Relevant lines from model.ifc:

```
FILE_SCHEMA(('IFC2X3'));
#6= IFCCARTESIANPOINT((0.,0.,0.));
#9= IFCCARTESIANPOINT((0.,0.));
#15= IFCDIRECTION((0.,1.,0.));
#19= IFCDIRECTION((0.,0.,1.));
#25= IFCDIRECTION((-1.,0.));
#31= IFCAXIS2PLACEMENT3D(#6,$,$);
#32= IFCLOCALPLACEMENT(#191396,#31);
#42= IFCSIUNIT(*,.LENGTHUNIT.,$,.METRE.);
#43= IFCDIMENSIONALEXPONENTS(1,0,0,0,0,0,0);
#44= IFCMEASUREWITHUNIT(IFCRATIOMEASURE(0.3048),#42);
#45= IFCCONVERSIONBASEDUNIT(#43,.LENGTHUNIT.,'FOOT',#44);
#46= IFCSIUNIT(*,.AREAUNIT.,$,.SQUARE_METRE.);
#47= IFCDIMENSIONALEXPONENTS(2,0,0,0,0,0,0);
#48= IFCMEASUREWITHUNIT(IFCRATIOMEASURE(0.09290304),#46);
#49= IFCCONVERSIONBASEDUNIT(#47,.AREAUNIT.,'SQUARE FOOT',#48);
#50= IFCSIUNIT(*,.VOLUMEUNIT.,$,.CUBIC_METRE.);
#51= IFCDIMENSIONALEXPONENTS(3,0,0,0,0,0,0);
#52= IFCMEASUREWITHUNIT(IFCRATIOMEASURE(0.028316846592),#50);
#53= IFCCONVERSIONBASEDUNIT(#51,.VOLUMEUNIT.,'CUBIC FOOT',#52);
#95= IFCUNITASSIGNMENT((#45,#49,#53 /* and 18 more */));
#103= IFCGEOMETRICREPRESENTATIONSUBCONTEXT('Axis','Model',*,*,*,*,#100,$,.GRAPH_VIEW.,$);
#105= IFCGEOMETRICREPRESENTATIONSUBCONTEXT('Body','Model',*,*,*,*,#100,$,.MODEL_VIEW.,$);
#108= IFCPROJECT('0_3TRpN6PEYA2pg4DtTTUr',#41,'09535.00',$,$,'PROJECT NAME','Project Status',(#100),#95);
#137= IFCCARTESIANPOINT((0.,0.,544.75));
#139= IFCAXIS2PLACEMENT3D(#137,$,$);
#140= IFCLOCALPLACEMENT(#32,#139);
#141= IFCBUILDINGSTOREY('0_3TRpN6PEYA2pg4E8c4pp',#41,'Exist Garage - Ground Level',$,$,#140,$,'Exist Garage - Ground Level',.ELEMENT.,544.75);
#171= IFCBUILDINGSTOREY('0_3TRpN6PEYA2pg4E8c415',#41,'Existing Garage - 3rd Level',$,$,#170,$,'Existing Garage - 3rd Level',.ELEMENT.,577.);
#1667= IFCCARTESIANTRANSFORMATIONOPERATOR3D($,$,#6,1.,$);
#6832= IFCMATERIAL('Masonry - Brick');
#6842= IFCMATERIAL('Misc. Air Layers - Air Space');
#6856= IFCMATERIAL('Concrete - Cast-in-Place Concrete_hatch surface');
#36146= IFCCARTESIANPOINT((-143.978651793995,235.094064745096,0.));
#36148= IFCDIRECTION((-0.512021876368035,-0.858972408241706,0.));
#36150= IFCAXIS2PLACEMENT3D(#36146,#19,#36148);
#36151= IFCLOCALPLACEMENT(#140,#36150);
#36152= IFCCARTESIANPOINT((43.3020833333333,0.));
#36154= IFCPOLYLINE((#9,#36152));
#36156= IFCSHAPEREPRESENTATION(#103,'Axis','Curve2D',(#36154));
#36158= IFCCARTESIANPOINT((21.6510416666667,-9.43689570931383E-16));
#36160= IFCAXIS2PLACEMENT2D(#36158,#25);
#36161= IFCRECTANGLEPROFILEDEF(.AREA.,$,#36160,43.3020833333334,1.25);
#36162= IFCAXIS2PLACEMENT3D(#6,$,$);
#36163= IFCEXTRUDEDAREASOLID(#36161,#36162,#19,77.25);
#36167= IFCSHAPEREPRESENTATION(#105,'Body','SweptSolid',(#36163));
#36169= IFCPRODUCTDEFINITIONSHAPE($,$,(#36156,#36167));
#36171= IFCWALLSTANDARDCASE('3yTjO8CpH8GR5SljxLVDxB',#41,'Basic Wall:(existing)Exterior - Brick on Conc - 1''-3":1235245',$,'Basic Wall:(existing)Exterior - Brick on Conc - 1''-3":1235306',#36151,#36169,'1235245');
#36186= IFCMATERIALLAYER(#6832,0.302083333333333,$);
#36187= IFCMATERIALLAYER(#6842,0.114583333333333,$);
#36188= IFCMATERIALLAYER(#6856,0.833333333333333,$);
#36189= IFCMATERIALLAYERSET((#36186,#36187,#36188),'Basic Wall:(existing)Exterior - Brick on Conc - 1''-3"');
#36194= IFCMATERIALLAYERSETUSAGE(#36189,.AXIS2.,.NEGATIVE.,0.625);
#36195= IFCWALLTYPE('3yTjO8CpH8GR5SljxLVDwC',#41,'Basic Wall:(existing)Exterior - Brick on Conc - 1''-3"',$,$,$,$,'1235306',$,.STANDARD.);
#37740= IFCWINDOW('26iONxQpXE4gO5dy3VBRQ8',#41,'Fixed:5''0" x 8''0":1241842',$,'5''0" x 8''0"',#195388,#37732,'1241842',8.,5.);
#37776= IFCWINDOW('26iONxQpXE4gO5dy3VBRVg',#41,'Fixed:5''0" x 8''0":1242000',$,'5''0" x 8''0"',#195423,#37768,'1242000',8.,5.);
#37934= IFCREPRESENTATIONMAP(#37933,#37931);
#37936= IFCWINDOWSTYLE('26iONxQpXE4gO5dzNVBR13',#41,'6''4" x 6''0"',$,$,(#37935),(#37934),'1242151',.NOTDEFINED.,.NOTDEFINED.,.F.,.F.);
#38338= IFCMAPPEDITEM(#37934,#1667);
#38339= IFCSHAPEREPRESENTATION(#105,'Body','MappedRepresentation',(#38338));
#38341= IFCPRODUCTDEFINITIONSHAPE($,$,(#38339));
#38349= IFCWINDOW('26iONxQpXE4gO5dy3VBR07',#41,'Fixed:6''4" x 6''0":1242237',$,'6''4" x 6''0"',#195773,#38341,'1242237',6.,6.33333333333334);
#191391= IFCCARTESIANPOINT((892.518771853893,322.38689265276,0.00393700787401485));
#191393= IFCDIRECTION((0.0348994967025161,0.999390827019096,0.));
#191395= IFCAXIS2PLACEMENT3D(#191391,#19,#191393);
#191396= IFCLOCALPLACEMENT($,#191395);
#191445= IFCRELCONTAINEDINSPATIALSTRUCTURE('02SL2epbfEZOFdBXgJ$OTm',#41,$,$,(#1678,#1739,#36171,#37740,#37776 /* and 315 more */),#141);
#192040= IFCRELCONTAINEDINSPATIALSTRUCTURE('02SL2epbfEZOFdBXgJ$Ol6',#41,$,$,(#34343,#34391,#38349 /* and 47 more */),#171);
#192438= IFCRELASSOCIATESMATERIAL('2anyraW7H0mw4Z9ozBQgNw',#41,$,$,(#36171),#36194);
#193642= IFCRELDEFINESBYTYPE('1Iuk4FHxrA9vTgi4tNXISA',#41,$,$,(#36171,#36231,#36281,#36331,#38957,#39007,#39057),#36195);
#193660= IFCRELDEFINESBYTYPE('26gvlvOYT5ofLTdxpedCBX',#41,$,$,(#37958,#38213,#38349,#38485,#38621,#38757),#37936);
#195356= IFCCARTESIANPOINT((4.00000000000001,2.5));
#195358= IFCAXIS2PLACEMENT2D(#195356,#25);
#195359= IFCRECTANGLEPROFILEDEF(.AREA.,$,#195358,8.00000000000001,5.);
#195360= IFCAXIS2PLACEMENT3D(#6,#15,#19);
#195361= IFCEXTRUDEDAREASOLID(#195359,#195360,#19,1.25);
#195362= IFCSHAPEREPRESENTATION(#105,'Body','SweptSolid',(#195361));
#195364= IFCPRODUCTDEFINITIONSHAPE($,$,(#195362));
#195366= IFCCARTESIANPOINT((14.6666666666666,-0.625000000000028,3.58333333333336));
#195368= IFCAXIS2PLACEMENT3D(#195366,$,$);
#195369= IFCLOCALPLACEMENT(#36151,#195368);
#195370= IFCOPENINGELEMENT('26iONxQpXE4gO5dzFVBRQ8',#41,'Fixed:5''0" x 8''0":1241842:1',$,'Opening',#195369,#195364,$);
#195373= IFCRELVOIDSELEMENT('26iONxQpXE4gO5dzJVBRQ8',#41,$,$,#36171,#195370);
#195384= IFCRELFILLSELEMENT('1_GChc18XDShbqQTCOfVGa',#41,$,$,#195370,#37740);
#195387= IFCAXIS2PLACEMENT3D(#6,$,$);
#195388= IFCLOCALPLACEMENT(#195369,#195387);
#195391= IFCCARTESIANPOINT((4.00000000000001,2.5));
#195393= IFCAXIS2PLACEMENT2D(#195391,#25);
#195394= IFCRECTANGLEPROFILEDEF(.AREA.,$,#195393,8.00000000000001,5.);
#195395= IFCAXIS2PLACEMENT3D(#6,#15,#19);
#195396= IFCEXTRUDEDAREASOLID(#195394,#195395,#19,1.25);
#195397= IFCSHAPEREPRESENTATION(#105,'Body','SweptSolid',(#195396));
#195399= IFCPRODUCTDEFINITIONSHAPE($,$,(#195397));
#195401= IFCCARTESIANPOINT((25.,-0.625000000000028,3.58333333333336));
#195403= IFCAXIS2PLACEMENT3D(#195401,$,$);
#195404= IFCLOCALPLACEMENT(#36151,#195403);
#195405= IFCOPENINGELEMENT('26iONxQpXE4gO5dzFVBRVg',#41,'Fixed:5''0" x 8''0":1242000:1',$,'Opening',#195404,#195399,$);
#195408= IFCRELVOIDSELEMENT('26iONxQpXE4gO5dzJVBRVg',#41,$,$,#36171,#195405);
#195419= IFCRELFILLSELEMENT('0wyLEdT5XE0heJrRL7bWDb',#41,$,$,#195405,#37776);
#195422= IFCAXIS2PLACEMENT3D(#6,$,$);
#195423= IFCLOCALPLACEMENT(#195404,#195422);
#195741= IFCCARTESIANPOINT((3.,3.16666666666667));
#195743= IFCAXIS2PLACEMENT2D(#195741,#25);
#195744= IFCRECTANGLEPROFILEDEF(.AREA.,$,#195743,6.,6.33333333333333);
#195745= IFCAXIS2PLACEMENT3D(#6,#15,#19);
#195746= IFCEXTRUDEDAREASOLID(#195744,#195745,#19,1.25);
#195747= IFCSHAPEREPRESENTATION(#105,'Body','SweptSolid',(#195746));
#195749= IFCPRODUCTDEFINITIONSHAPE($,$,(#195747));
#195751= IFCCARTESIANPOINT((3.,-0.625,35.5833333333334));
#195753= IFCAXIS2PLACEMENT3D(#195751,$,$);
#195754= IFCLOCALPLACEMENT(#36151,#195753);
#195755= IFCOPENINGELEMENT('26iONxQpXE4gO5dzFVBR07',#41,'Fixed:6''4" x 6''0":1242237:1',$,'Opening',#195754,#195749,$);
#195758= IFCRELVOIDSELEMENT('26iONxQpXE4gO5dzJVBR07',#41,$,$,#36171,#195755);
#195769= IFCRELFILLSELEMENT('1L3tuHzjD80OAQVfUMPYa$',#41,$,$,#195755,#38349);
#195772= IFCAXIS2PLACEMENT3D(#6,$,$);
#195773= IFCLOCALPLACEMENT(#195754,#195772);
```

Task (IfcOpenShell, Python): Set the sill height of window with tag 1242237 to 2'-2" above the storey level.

```python
import numpy as np
import ifcopenshell
import ifcopenshell.api.geometry
import ifcopenshell.geom
import ifcopenshell.util.element
import ifcopenshell.util.placement
import ifcopenshell.util.shape
import ifcopenshell.util.unit

model = ifcopenshell.open("model.ifc")
unit_scale = ifcopenshell.util.unit.calculate_unit_scale(model)

window = model.by_guid("26iONxQpXE4gO5dy3VBR07")
opening = window.FillsVoids[0].RelatingOpeningElement
storey = ifcopenshell.util.element.get_container(window, ifc_class="IfcBuildingStorey")
level = ifcopenshell.util.placement.get_local_placement(storey.ObjectPlacement)[2, 3]

# The opening's origin need not be at the sill, so measure its lowest point.
shape = ifcopenshell.geom.create_shape(ifcopenshell.geom.settings(), opening)
bottom = ifcopenshell.util.shape.get_shape_bottom_elevation(shape, shape.geometry) / unit_scale
dz = level + 26 * 0.0254 / unit_scale - bottom

shift = np.array([0.0, 0.0, dz])
# The window is placed relative to its opening, so it follows when the opening moves.
matrix = ifcopenshell.util.placement.get_local_placement(opening.ObjectPlacement)
matrix[:3, 3] += shift
ifcopenshell.api.geometry.edit_object_placement(
    model, product=opening, matrix=matrix, is_si=False, should_transform_children=True
)

print(f"moved by {dz * unit_scale:+.3f} m")

model.write("model_v2.ifc")
```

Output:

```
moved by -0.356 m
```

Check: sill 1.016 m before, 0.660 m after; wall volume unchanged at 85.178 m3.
